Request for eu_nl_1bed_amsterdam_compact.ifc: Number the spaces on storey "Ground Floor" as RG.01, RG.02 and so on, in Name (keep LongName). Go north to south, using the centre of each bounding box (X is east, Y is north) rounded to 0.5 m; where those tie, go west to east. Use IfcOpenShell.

First a look at what the model holds.

```python
import ifcopenshell
import ifcopenshell.util.element
import ifcopenshell.util.placement

model = ifcopenshell.open("eu_nl_1bed_amsterdam_compact.ifc")
print(model.schema)
storey = next(s for s in model.by_type("IfcBuildingStorey") if s.Name == "Ground Floor")
spaces = [e for e in ifcopenshell.util.element.get_decomposition(storey) if e.is_a("IfcSpace")]
for e in sorted(spaces, key=lambda e: e.id()):
    origin = ifcopenshell.util.placement.get_local_placement(e.ObjectPlacement)[:3, 3]
    print(e.id(), e.Name, e.LongName, origin.round(2) + 0.0, sep=" | ")
```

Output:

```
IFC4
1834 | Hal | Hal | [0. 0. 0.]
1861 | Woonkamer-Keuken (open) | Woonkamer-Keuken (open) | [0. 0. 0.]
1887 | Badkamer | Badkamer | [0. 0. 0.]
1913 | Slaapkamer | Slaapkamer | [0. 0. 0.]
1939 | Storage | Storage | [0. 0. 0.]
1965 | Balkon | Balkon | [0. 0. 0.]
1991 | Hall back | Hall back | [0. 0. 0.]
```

```python
import ifcopenshell
import ifcopenshell.geom
import ifcopenshell.util.element
import ifcopenshell.util.shape

model = ifcopenshell.open("eu_nl_1bed_amsterdam_compact.ifc")
settings = ifcopenshell.geom.settings()
settings.set("use-world-coords", True)


def centre(element):
    shape = ifcopenshell.geom.create_shape(settings, element)
    return ifcopenshell.util.shape.get_bbox_centroid(shape.geometry)


storey = next(s for s in model.by_type("IfcBuildingStorey") if s.Name == "Ground Floor")
spaces = [e for e in ifcopenshell.util.element.get_decomposition(storey) if e.is_a("IfcSpace")]

# Insertion points can sit at a corner or the storey origin, so sort by the geometry (in metres).
centres = {e: centre(e) for e in spaces}
spaces.sort(key=lambda e: (-round(centres[e][1] / 0.5), centres[e][0]))

for i, e in enumerate(spaces, start=1):
    number = f"RG.{i:02d}"
    e.Name = number
    print(e.id(), number)

model.write("eu_nl_1bed_amsterdam_compact_v2.ifc")
```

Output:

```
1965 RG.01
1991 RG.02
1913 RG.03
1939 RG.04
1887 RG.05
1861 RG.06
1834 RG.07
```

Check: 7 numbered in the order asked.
